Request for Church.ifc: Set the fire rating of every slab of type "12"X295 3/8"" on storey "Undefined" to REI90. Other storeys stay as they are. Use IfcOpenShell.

First a look at what the model holds.

```python
import ifcopenshell
import ifcopenshell.util.element

model = ifcopenshell.open("Church.ifc")
print(model.schema)
storey = next(s for s in model.by_type("IfcBuildingStorey") if s.Name == "Undefined")
slabs = [e for e in ifcopenshell.util.element.get_decomposition(storey) if e.is_a("IfcSlab")]
seen = {}
for e in slabs:
    element_type = ifcopenshell.util.element.get_type(e)
    key = (element_type.Name if element_type != e and element_type else None, ifcopenshell.util.element.get_pset(e, "Pset_SlabCommon", "FireRating"))
    seen[key] = seen.get(key, 0) + 1
for (name, value), count in sorted(seen.items(), key=str):
    print(count, "x", name, "|", value)
```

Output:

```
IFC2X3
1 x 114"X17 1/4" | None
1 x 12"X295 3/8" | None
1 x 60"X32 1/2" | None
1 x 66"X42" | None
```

```python
import ifcopenshell
import ifcopenshell.api.pset
import ifcopenshell.util.element

model = ifcopenshell.open("Church.ifc")

storey = next(s for s in model.by_type("IfcBuildingStorey") if s.Name == "Undefined")
slabs = [e for e in ifcopenshell.util.element.get_decomposition(storey) if e.is_a("IfcSlab")]

count = 0
for e in slabs:
    element_type = ifcopenshell.util.element.get_type(e)
    if element_type in (None, e) or element_type.Name != '12"X295 3/8"':
        continue
    # add_pset returns the element's existing set when there is one.
    pset = ifcopenshell.api.pset.add_pset(model, product=e, name="Pset_SlabCommon")
    ifcopenshell.api.pset.edit_pset(model, pset=pset, properties={"FireRating": "REI90"})
    count += 1

print(count, "slabs updated")

model.write("Church_edited.ifc")
```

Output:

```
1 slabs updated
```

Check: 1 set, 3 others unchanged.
